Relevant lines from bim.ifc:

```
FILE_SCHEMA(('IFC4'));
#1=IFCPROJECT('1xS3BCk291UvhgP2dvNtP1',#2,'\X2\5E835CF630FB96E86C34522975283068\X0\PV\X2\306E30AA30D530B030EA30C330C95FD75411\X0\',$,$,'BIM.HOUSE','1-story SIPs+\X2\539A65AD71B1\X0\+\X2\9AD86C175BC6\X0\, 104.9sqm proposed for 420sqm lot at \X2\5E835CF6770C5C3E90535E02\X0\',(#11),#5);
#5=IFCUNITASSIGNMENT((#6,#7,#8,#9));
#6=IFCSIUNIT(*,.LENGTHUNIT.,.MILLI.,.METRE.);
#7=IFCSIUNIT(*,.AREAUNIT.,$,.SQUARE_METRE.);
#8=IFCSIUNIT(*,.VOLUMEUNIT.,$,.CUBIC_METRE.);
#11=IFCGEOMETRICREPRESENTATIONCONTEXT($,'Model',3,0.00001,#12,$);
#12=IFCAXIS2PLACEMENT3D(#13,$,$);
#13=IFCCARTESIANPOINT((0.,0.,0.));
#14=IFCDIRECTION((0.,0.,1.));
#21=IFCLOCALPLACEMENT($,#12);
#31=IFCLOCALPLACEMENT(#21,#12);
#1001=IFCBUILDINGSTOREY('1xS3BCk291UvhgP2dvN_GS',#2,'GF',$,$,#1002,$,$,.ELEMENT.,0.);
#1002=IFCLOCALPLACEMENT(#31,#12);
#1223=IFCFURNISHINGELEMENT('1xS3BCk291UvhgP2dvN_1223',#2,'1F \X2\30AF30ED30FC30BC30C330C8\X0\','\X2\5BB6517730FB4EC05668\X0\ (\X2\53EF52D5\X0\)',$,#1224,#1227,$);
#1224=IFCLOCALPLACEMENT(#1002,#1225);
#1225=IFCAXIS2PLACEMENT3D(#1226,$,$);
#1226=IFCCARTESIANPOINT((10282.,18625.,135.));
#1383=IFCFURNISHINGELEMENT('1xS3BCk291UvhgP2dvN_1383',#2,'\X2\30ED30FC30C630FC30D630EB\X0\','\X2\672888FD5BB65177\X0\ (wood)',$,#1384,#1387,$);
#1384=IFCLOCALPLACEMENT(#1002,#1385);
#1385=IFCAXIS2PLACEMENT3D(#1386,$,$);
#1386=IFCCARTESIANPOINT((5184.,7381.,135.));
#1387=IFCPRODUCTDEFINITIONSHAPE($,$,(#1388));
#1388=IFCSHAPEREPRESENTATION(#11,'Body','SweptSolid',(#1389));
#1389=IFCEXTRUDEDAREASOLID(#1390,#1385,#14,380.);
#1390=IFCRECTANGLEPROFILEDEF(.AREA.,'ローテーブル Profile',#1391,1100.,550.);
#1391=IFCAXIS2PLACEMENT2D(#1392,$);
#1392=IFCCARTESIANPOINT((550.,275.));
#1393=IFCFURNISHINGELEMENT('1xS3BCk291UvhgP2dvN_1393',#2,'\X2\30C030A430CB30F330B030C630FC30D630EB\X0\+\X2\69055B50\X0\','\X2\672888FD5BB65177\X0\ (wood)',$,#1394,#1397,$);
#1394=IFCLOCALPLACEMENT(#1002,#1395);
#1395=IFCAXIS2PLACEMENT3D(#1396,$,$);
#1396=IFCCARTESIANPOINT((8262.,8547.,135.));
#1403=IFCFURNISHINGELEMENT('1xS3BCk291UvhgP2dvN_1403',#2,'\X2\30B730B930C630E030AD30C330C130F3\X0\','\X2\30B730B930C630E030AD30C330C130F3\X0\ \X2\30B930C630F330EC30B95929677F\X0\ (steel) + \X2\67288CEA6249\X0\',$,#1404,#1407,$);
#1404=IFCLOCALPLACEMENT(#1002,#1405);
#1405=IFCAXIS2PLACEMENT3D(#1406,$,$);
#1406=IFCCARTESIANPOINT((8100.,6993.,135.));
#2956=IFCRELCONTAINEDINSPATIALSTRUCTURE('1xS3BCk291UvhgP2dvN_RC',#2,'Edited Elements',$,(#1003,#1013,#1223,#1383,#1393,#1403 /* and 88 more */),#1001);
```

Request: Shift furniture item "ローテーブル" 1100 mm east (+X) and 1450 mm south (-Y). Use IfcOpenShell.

```python
import ifcopenshell
import ifcopenshell.api.geometry
import ifcopenshell.util.placement
import ifcopenshell.util.unit

model = ifcopenshell.open("bim.ifc")
unit_scale = ifcopenshell.util.unit.calculate_unit_scale(model)

item = model.by_guid("1xS3BCk291UvhgP2dvN_1383")
matrix = ifcopenshell.util.placement.get_local_placement(item.ObjectPlacement)
matrix[0, 3] += 1.1 / unit_scale
matrix[1, 3] -= 1.45 / unit_scale
ifcopenshell.api.geometry.edit_object_placement(model, product=item, matrix=matrix, is_si=False)

print(ifcopenshell.util.placement.get_local_placement(item.ObjectPlacement).round(3) + 0.0)

model.write("bim-out.ifc")
```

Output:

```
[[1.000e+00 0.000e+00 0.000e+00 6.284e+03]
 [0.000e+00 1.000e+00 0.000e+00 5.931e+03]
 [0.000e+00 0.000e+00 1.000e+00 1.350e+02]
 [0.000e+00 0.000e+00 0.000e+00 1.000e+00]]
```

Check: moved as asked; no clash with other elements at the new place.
